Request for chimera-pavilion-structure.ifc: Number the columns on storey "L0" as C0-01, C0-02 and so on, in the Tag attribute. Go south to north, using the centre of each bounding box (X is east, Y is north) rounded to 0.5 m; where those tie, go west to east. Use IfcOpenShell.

First a look at what the model holds.

```python
import ifcopenshell
import ifcopenshell.util.element
import ifcopenshell.util.placement

model = ifcopenshell.open("chimera-pavilion-structure.ifc")
print(model.schema)
storey = next(s for s in model.by_type("IfcBuildingStorey") if s.Name == "L0")
columns = [e for e in ifcopenshell.util.element.get_decomposition(storey) if e.is_a("IfcColumn")]
for e in sorted(columns, key=lambda e: e.id()):
    origin = ifcopenshell.util.placement.get_local_placement(e.ObjectPlacement)[:3, 3]
    print(e.id(), e.Tag, e.Name, origin.round(2) + 0.0, sep=" | ")
```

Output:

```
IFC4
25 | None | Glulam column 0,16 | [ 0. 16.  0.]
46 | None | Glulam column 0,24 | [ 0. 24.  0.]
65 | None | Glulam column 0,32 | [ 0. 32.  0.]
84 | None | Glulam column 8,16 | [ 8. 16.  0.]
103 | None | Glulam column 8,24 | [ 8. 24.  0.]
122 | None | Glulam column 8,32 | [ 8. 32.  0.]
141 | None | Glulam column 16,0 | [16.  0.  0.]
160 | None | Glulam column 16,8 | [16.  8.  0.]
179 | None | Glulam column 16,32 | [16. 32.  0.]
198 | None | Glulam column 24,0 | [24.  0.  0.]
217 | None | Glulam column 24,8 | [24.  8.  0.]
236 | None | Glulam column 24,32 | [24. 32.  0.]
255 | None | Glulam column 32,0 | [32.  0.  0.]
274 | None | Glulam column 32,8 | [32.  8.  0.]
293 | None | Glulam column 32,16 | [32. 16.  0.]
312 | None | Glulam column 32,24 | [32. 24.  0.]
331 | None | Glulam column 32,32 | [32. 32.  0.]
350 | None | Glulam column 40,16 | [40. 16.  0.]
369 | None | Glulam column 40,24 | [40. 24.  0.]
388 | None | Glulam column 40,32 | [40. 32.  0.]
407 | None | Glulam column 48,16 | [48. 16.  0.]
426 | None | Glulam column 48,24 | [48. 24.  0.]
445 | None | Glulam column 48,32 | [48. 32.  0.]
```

```python
import ifcopenshell
import ifcopenshell.geom
import ifcopenshell.util.element
import ifcopenshell.util.shape

model = ifcopenshell.open("chimera-pavilion-structure.ifc")
settings = ifcopenshell.geom.settings()
settings.set("use-world-coords", True)


def centre(element):
    shape = ifcopenshell.geom.create_shape(settings, element)
    return ifcopenshell.util.shape.get_bbox_centroid(shape.geometry)


storey = next(s for s in model.by_type("IfcBuildingStorey") if s.Name == "L0")
columns = [e for e in ifcopenshell.util.element.get_decomposition(storey) if e.is_a("IfcColumn")]

# Insertion points can sit at a corner or the storey origin, so sort by the geometry (in metres).
centres = {e: centre(e) for e in columns}
columns.sort(key=lambda e: (round(centres[e][1] / 0.5), centres[e][0]))

for i, e in enumerate(columns, start=1):
    number = f"C0-{i:02d}"
    e.Tag = number
    print(e.id(), number)

model.write("chimera-pavilion-structure_updated.ifc")
```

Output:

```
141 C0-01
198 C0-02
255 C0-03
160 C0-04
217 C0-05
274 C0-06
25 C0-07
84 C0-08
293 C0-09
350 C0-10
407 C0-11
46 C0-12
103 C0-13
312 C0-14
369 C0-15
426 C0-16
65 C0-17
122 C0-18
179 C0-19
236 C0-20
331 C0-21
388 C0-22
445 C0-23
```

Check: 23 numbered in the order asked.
